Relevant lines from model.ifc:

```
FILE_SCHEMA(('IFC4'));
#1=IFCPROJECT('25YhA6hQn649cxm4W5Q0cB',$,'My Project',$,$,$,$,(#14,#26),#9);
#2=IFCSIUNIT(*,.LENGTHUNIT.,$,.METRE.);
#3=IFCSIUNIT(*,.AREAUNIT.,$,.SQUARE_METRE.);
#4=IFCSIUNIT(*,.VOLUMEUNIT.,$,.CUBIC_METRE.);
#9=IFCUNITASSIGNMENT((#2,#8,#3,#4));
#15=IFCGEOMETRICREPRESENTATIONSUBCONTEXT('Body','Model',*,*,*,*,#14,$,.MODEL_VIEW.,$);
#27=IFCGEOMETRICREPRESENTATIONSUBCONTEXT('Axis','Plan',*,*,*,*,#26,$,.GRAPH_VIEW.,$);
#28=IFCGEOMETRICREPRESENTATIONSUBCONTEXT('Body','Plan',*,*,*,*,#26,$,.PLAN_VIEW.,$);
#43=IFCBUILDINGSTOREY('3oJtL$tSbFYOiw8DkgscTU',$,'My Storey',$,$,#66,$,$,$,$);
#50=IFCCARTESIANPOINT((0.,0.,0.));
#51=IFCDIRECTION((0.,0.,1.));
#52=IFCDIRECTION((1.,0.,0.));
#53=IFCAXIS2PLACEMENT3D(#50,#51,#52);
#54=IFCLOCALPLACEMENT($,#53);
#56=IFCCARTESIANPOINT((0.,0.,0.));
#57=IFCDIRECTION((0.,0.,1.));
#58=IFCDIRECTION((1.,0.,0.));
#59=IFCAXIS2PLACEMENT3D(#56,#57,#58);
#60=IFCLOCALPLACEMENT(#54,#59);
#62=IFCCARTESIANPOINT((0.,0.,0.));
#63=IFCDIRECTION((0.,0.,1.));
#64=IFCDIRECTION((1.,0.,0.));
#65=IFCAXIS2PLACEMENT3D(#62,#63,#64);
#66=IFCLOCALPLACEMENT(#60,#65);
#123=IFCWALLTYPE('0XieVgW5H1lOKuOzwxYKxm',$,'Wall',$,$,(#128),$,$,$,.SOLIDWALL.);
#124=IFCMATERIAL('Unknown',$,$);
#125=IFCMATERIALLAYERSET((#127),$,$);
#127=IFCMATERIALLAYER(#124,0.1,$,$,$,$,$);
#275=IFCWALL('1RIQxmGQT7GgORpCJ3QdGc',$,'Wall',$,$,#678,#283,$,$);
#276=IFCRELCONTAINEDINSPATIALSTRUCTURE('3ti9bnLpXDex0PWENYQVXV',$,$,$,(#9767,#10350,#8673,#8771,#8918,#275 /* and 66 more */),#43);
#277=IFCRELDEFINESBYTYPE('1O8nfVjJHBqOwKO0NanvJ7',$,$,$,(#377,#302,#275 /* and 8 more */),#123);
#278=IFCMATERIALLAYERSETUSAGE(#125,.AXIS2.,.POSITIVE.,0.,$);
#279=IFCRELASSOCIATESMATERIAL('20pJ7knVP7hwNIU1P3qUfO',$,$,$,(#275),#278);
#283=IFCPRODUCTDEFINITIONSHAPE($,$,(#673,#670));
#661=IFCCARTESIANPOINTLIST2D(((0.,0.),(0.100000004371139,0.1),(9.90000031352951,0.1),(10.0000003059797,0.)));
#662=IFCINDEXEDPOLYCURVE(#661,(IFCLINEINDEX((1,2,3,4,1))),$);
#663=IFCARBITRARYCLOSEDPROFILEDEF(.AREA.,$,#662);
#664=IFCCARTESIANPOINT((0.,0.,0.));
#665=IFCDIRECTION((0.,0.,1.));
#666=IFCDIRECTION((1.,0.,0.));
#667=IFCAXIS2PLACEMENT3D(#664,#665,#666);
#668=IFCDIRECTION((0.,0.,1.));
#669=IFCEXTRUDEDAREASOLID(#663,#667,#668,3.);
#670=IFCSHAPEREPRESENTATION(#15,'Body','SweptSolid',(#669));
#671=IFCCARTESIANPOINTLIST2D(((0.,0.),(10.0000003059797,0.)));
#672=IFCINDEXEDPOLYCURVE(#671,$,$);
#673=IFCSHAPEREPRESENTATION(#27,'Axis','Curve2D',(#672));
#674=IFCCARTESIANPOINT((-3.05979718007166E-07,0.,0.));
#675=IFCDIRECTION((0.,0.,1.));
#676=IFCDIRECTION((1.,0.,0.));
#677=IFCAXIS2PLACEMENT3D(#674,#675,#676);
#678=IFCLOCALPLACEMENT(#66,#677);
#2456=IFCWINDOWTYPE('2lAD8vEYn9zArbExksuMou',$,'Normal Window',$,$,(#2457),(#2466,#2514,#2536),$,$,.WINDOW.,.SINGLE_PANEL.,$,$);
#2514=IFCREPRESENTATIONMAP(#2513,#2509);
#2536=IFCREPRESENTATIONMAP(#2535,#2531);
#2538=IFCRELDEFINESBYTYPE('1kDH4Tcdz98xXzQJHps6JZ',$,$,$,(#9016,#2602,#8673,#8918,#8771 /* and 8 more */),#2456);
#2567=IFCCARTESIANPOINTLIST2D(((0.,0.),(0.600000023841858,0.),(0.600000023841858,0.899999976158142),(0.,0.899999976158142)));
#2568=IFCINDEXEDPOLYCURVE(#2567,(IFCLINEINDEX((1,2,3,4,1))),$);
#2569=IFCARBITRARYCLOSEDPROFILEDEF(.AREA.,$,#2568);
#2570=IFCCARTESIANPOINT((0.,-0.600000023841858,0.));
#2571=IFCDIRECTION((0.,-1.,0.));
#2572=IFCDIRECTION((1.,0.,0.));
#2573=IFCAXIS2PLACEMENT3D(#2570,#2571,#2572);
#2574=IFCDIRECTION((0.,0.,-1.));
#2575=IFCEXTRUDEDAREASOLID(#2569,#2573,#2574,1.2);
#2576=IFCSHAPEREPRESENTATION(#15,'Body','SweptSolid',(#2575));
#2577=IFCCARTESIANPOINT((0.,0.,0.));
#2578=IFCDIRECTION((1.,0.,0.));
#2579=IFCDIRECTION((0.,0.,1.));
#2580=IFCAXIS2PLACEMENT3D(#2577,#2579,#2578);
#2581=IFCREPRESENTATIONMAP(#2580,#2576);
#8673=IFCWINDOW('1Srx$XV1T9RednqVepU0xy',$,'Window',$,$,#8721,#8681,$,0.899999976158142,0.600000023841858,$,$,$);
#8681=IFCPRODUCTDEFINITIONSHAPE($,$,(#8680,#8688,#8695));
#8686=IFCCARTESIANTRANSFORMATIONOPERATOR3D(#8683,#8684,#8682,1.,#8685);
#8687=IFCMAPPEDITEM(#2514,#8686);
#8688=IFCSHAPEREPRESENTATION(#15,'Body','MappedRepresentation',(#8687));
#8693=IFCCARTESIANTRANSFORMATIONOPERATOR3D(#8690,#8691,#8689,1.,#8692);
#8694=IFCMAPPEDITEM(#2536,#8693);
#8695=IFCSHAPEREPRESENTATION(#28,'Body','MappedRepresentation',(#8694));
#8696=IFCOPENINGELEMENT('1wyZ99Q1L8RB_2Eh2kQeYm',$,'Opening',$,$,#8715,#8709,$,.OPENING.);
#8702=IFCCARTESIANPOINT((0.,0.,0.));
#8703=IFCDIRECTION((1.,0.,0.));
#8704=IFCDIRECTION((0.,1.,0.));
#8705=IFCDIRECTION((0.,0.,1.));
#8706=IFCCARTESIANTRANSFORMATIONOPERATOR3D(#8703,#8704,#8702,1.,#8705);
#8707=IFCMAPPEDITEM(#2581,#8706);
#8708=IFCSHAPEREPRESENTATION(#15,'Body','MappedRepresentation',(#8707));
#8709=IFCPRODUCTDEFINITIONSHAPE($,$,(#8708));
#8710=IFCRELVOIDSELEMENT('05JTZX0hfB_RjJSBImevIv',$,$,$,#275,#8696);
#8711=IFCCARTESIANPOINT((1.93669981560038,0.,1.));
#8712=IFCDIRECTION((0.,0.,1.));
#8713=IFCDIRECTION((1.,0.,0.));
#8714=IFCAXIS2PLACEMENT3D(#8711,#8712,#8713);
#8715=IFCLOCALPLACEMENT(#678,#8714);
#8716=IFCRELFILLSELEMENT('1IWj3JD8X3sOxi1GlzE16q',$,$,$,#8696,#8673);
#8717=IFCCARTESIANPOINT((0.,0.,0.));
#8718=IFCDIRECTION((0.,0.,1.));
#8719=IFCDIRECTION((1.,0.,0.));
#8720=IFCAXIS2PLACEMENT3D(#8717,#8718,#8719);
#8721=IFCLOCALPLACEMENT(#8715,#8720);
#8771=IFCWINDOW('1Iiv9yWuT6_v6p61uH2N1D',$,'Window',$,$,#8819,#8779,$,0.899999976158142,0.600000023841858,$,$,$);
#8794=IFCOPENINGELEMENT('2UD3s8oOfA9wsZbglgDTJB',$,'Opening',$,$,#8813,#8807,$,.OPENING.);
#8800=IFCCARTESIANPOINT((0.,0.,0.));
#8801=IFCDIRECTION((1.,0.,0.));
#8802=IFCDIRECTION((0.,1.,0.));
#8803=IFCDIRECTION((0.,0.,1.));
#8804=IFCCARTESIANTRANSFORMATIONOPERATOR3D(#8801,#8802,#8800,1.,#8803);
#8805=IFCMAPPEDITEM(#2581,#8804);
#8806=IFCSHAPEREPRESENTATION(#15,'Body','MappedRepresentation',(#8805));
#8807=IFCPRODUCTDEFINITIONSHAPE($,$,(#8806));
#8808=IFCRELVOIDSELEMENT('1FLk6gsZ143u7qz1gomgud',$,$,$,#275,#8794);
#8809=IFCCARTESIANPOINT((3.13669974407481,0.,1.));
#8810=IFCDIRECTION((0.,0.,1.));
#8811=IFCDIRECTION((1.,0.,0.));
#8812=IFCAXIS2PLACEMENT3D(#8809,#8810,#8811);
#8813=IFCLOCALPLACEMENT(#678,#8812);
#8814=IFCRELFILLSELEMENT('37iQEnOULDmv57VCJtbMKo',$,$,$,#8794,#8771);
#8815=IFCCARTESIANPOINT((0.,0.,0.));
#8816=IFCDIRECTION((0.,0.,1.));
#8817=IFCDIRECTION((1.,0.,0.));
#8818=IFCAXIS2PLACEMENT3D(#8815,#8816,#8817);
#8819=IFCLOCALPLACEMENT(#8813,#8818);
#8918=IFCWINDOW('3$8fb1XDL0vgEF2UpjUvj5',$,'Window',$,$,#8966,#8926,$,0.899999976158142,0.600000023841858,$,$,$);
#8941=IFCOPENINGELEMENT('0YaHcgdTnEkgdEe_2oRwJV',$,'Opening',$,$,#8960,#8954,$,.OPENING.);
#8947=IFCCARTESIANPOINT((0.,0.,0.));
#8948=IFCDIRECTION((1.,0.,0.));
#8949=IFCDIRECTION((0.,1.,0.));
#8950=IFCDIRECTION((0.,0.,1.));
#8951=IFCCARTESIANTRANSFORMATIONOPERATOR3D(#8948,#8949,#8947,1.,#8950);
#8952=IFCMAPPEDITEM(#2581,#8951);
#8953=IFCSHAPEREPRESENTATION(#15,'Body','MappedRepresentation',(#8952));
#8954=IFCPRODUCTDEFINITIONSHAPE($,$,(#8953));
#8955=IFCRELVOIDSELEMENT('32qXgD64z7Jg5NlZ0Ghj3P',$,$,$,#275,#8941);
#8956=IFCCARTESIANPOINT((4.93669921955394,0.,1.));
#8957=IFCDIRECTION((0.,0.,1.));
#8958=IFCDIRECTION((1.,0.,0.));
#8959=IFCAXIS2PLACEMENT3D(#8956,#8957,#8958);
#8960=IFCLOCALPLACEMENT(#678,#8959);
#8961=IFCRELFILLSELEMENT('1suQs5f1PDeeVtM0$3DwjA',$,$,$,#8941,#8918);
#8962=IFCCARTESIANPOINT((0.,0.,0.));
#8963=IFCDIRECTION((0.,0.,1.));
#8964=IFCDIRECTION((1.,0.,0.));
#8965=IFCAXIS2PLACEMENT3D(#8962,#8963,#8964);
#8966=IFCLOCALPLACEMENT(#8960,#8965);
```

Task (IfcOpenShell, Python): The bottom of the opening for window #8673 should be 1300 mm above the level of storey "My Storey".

```python
import numpy as np
import ifcopenshell
import ifcopenshell.api.geometry
import ifcopenshell.geom
import ifcopenshell.util.element
import ifcopenshell.util.placement
import ifcopenshell.util.shape
import ifcopenshell.util.unit

model = ifcopenshell.open("model.ifc")
unit_scale = ifcopenshell.util.unit.calculate_unit_scale(model)

window = model.by_id(8673)
opening = window.FillsVoids[0].RelatingOpeningElement
storey = ifcopenshell.util.element.get_container(window, ifc_class="IfcBuildingStorey")
level = ifcopenshell.util.placement.get_local_placement(storey.ObjectPlacement)[2, 3]

# The opening's origin need not be at the sill, so measure its lowest point.
shape = ifcopenshell.geom.create_shape(ifcopenshell.geom.settings(), opening)
bottom = ifcopenshell.util.shape.get_shape_bottom_elevation(shape, shape.geometry) / unit_scale
dz = level + 1.3 - bottom

shift = np.array([0.0, 0.0, dz])
# The window is placed relative to its opening, so it follows when the opening moves.
matrix = ifcopenshell.util.placement.get_local_placement(opening.ObjectPlacement)
matrix[:3, 3] += shift
ifcopenshell.api.geometry.edit_object_placement(
    model, product=opening, matrix=matrix, is_si=False, should_transform_children=True
)

print(f"moved by {dz * unit_scale:+.3f} m")

model.write("model-out.ifc")
```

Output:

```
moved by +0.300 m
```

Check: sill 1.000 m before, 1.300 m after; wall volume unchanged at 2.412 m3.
